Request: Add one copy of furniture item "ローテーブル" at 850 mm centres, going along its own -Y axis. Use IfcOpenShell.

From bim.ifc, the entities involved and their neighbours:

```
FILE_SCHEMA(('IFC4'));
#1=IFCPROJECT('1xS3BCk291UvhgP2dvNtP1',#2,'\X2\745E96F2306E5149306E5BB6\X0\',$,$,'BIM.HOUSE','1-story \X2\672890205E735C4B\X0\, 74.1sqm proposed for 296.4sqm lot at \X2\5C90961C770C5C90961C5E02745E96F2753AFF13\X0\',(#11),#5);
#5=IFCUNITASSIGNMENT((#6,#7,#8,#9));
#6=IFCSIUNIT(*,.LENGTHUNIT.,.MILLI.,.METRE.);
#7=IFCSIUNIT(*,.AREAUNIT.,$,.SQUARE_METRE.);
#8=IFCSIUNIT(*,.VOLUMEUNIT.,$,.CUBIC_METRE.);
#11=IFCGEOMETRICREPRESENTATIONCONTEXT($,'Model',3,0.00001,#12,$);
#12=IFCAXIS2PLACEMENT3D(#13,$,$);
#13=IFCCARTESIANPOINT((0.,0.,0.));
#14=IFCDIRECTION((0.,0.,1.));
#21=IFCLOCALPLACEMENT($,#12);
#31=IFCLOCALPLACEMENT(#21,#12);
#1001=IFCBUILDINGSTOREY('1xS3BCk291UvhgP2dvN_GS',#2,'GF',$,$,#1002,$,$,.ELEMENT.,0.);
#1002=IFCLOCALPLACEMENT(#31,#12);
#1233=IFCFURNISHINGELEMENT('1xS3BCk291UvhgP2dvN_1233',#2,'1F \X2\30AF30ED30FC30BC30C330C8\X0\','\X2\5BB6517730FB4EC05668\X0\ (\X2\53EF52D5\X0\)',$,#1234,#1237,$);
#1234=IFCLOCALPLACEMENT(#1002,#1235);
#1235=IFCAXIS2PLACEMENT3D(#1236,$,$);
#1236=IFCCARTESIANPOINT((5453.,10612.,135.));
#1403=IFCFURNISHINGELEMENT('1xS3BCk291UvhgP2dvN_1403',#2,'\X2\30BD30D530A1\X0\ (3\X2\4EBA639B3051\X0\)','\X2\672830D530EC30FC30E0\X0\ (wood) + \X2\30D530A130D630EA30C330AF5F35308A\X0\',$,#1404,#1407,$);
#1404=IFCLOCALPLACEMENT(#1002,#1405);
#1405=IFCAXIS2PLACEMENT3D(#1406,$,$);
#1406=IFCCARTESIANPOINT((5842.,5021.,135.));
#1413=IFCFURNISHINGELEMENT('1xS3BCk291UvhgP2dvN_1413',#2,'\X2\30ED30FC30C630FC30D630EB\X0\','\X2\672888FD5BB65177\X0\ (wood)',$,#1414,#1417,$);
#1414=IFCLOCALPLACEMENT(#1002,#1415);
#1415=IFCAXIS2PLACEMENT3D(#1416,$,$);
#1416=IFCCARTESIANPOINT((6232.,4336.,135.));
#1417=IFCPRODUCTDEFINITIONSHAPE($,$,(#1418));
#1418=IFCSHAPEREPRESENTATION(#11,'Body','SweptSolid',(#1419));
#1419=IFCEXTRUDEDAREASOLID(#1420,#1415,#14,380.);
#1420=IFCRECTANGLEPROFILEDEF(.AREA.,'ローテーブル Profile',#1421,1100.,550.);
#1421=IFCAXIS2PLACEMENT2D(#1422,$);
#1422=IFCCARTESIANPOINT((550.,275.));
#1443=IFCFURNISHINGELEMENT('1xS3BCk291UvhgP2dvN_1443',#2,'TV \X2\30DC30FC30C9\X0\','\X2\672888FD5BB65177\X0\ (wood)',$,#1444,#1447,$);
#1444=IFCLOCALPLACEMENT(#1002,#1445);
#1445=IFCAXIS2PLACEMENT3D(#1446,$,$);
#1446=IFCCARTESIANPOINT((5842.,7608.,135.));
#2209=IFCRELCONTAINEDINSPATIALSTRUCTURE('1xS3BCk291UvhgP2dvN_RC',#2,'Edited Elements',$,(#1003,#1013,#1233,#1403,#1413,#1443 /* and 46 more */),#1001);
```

```python
import ifcopenshell
import ifcopenshell.api.geometry
import ifcopenshell.api.root
import ifcopenshell.util.element
import ifcopenshell.util.placement

model = ifcopenshell.open("bim.ifc")


def reuse_history(source, copy):
    """copy_class also copies each property set's owner history, people and application; keep the originals."""
    for rel in copy.IsDefinedBy:
        if rel.is_a("IfcRelDefinesByProperties") and (history := rel.RelatingPropertyDefinition.OwnerHistory):
            rel.RelatingPropertyDefinition.OwnerHistory = source.OwnerHistory
            ifcopenshell.util.element.remove_deep2(model, history)


source = model.by_id(1413)
base = ifcopenshell.util.placement.get_local_placement(source.ObjectPlacement)
step = -base[:3, 1] * 850.0

for i in range(1, 2):
    copy = ifcopenshell.api.root.copy_class(model, product=source)
    copy.Representation = ifcopenshell.util.element.copy_deep(
        model, source.Representation, exclude=["IfcGeometricRepresentationContext", "IfcRepresentationMap"]
    )
    reuse_history(source, copy)
    matrix = base.copy()
    matrix[:3, 3] += i * step
    print("added at", matrix[:3, 3].round(3) + 0.0)
    ifcopenshell.api.geometry.edit_object_placement(model, product=copy, matrix=matrix, is_si=False)

model.write("bim_rev.ifc")
```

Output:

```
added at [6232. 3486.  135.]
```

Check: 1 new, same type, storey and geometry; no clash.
